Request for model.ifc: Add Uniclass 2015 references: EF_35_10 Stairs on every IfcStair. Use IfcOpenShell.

First a look at what the model holds.

```python
import ifcopenshell

model = ifcopenshell.open("model.ifc")
print(model.schema)
print("classifications:", [c.Name for c in model.by_type("IfcClassification")])
for ifc_class in ("IfcDoor", "IfcRoof", "IfcStair", "IfcWall", "IfcWindow"):
    print(ifc_class, len(model.by_type(ifc_class)))
```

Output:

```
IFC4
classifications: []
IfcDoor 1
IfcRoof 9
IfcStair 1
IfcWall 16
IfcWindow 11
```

```python
import ifcopenshell
import ifcopenshell.api.classification

model = ifcopenshell.open("model.ifc")

system = ifcopenshell.api.classification.add_classification(model, classification="Uniclass 2015")

codes = {
    "IfcStair": ("EF_35_10", "Stairs"),
}
for ifc_class, (code, name) in codes.items():
    products = model.by_type(ifc_class)
    ifcopenshell.api.classification.add_reference(
        model, products=products, classification=system, identification=code, name=name
    )
    print(code, len(products))

model.write("model-out.ifc")
```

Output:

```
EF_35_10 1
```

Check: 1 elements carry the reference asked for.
